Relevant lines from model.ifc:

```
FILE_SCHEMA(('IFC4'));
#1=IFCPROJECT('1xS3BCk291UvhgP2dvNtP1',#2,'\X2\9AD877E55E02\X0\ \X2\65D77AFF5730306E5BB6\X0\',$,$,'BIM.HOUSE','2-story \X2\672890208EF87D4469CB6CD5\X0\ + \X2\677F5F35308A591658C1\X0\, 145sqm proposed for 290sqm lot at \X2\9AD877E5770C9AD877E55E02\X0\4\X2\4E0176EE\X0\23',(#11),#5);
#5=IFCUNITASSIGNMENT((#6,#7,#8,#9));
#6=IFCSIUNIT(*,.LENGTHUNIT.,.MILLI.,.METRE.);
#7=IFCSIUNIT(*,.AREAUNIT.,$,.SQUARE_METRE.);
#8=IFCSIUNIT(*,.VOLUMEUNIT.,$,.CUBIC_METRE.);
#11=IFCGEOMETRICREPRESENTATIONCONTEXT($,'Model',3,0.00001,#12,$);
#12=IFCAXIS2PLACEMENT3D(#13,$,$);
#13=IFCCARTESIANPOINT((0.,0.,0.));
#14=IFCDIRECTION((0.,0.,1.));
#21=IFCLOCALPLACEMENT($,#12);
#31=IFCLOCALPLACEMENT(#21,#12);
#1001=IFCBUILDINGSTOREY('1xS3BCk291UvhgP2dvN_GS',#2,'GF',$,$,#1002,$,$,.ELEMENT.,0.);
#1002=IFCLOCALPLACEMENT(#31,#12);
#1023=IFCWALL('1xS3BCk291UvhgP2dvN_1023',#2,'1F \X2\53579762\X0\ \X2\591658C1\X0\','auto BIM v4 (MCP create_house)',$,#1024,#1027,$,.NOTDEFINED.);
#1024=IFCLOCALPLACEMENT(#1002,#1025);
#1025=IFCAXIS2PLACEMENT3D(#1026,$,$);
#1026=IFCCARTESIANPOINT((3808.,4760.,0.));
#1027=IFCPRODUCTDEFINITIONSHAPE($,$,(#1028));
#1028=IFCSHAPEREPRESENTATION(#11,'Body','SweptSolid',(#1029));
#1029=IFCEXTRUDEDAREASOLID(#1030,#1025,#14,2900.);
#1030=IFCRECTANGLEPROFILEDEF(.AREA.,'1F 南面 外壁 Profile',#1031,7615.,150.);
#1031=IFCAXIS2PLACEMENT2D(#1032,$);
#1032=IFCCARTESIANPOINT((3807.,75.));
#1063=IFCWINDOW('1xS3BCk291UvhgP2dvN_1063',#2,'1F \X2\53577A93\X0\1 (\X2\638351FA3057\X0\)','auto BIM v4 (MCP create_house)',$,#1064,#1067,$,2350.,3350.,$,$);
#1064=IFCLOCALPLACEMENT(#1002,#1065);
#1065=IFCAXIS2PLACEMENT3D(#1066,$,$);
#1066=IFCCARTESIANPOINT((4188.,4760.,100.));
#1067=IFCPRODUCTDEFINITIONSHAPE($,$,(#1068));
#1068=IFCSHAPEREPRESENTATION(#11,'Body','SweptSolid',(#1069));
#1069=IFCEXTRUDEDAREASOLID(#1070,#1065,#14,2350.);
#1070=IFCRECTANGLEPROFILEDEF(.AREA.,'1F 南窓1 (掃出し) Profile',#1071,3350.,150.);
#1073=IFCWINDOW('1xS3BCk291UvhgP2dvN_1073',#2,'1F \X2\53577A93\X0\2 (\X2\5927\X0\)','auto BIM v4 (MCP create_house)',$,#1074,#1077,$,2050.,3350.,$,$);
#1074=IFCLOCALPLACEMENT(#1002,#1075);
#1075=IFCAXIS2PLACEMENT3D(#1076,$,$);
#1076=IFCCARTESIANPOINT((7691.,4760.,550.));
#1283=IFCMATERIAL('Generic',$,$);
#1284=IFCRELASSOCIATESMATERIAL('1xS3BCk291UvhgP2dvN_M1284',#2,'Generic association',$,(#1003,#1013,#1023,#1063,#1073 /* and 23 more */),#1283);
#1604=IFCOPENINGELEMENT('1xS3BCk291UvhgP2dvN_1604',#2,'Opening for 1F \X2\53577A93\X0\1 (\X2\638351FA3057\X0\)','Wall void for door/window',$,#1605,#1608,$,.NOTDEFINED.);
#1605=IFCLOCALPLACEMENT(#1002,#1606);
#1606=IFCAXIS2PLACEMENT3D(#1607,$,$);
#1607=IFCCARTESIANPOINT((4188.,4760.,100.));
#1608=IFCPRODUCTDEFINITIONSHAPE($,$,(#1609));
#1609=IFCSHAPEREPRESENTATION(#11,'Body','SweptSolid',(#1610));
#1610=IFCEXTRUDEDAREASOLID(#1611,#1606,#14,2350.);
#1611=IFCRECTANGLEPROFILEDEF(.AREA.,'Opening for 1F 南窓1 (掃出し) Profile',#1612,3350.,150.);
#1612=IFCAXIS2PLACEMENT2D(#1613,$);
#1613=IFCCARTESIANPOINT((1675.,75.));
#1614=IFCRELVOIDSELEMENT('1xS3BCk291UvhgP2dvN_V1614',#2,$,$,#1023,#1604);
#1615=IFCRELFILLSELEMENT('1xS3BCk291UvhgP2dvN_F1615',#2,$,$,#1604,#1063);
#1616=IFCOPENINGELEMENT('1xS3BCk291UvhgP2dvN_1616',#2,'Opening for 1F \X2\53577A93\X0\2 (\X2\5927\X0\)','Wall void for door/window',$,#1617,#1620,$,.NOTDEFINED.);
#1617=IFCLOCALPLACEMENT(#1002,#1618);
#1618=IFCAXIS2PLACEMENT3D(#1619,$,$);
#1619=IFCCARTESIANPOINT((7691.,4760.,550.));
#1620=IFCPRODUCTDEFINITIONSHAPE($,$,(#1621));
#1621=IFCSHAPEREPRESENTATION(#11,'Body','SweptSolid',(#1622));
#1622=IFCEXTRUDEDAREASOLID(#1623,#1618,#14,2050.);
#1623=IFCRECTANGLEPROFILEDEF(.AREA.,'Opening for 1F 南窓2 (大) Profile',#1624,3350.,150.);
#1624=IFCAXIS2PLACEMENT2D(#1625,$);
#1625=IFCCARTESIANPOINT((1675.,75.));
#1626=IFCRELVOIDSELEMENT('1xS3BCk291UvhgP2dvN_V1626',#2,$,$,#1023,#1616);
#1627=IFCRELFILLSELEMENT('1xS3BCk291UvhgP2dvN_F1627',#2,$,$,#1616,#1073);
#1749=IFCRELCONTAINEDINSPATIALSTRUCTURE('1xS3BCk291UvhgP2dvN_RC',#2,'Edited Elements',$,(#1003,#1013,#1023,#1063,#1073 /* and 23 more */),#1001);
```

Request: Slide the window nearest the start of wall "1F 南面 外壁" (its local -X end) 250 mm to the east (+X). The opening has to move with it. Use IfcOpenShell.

```python
import ifcopenshell
import ifcopenshell.api.geometry
import ifcopenshell.util.placement
import ifcopenshell.util.unit

model = ifcopenshell.open("model.ifc")
unit_scale = ifcopenshell.util.unit.calculate_unit_scale(model)

window = model.by_guid("1xS3BCk291UvhgP2dvN_1063")
opening = window.FillsVoids[0].RelatingOpeningElement
wall = opening.VoidsElements[0].RelatingBuildingElement

wall_matrix = ifcopenshell.util.placement.get_local_placement(wall.ObjectPlacement)
shift = wall_matrix[:3, 0] * 0.25 / unit_scale
before = ifcopenshell.util.placement.get_local_placement(window.ObjectPlacement)[:3, 3].copy()

# The window is not placed relative to its opening, so move both.
for product in (opening, window):
    matrix = ifcopenshell.util.placement.get_local_placement(product.ObjectPlacement)
    matrix[:3, 3] += shift
    ifcopenshell.api.geometry.edit_object_placement(model, product=product, matrix=matrix, is_si=False)

after = ifcopenshell.util.placement.get_local_placement(window.ObjectPlacement)[:3, 3]
print("window moved by", (after - before).round(3) + 0.0)

model.write("model_v2.ifc")
```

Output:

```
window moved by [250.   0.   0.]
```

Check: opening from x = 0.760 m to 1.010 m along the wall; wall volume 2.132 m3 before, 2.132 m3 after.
